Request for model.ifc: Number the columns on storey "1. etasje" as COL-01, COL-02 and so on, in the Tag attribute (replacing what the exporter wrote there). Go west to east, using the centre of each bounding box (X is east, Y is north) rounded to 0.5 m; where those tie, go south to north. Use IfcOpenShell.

First a look at what the model holds.

```python
import ifcopenshell
import ifcopenshell.util.element
import ifcopenshell.util.placement

model = ifcopenshell.open("model.ifc")
print(model.schema)
storey = next(s for s in model.by_type("IfcBuildingStorey") if s.Name == "1. etasje")
columns = [e for e in ifcopenshell.util.element.get_decomposition(storey) if e.is_a("IfcColumn")]
for e in sorted(columns, key=lambda e: e.id()):
    origin = ifcopenshell.util.placement.get_local_placement(e.ObjectPlacement)[:3, 3]
    print(e.id(), e.Tag, e.Name, origin.round(2) + 0.0, sep=" | ")
```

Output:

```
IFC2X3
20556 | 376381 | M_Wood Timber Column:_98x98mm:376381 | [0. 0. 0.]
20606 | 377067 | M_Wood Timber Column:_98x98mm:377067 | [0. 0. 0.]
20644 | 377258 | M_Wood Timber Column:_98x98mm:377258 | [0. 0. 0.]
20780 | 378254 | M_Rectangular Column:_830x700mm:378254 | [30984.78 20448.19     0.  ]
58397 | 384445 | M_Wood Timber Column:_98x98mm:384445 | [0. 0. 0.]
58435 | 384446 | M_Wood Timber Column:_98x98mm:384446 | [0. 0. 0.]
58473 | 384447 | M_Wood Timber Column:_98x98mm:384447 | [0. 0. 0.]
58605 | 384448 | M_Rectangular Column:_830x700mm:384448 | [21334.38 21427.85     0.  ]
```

```python
import ifcopenshell
import ifcopenshell.geom
import ifcopenshell.util.element
import ifcopenshell.util.shape

model = ifcopenshell.open("model.ifc")
settings = ifcopenshell.geom.settings()
settings.set("use-world-coords", True)


def centre(element):
    shape = ifcopenshell.geom.create_shape(settings, element)
    return ifcopenshell.util.shape.get_bbox_centroid(shape.geometry)


storey = next(s for s in model.by_type("IfcBuildingStorey") if s.Name == "1. etasje")
columns = [e for e in ifcopenshell.util.element.get_decomposition(storey) if e.is_a("IfcColumn")]

# Insertion points can sit at a corner or the storey origin, so sort by the geometry (in metres).
centres = {e: centre(e) for e in columns}
columns.sort(key=lambda e: (round(centres[e][0] / 0.5), centres[e][1]))

for i, e in enumerate(columns, start=1):
    number = f"COL-{i:02d}"
    e.Tag = number
    print(e.id(), number)

model.write("model_edited.ifc")
```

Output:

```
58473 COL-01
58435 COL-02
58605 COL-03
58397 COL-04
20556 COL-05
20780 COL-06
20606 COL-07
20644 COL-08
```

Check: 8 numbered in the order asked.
